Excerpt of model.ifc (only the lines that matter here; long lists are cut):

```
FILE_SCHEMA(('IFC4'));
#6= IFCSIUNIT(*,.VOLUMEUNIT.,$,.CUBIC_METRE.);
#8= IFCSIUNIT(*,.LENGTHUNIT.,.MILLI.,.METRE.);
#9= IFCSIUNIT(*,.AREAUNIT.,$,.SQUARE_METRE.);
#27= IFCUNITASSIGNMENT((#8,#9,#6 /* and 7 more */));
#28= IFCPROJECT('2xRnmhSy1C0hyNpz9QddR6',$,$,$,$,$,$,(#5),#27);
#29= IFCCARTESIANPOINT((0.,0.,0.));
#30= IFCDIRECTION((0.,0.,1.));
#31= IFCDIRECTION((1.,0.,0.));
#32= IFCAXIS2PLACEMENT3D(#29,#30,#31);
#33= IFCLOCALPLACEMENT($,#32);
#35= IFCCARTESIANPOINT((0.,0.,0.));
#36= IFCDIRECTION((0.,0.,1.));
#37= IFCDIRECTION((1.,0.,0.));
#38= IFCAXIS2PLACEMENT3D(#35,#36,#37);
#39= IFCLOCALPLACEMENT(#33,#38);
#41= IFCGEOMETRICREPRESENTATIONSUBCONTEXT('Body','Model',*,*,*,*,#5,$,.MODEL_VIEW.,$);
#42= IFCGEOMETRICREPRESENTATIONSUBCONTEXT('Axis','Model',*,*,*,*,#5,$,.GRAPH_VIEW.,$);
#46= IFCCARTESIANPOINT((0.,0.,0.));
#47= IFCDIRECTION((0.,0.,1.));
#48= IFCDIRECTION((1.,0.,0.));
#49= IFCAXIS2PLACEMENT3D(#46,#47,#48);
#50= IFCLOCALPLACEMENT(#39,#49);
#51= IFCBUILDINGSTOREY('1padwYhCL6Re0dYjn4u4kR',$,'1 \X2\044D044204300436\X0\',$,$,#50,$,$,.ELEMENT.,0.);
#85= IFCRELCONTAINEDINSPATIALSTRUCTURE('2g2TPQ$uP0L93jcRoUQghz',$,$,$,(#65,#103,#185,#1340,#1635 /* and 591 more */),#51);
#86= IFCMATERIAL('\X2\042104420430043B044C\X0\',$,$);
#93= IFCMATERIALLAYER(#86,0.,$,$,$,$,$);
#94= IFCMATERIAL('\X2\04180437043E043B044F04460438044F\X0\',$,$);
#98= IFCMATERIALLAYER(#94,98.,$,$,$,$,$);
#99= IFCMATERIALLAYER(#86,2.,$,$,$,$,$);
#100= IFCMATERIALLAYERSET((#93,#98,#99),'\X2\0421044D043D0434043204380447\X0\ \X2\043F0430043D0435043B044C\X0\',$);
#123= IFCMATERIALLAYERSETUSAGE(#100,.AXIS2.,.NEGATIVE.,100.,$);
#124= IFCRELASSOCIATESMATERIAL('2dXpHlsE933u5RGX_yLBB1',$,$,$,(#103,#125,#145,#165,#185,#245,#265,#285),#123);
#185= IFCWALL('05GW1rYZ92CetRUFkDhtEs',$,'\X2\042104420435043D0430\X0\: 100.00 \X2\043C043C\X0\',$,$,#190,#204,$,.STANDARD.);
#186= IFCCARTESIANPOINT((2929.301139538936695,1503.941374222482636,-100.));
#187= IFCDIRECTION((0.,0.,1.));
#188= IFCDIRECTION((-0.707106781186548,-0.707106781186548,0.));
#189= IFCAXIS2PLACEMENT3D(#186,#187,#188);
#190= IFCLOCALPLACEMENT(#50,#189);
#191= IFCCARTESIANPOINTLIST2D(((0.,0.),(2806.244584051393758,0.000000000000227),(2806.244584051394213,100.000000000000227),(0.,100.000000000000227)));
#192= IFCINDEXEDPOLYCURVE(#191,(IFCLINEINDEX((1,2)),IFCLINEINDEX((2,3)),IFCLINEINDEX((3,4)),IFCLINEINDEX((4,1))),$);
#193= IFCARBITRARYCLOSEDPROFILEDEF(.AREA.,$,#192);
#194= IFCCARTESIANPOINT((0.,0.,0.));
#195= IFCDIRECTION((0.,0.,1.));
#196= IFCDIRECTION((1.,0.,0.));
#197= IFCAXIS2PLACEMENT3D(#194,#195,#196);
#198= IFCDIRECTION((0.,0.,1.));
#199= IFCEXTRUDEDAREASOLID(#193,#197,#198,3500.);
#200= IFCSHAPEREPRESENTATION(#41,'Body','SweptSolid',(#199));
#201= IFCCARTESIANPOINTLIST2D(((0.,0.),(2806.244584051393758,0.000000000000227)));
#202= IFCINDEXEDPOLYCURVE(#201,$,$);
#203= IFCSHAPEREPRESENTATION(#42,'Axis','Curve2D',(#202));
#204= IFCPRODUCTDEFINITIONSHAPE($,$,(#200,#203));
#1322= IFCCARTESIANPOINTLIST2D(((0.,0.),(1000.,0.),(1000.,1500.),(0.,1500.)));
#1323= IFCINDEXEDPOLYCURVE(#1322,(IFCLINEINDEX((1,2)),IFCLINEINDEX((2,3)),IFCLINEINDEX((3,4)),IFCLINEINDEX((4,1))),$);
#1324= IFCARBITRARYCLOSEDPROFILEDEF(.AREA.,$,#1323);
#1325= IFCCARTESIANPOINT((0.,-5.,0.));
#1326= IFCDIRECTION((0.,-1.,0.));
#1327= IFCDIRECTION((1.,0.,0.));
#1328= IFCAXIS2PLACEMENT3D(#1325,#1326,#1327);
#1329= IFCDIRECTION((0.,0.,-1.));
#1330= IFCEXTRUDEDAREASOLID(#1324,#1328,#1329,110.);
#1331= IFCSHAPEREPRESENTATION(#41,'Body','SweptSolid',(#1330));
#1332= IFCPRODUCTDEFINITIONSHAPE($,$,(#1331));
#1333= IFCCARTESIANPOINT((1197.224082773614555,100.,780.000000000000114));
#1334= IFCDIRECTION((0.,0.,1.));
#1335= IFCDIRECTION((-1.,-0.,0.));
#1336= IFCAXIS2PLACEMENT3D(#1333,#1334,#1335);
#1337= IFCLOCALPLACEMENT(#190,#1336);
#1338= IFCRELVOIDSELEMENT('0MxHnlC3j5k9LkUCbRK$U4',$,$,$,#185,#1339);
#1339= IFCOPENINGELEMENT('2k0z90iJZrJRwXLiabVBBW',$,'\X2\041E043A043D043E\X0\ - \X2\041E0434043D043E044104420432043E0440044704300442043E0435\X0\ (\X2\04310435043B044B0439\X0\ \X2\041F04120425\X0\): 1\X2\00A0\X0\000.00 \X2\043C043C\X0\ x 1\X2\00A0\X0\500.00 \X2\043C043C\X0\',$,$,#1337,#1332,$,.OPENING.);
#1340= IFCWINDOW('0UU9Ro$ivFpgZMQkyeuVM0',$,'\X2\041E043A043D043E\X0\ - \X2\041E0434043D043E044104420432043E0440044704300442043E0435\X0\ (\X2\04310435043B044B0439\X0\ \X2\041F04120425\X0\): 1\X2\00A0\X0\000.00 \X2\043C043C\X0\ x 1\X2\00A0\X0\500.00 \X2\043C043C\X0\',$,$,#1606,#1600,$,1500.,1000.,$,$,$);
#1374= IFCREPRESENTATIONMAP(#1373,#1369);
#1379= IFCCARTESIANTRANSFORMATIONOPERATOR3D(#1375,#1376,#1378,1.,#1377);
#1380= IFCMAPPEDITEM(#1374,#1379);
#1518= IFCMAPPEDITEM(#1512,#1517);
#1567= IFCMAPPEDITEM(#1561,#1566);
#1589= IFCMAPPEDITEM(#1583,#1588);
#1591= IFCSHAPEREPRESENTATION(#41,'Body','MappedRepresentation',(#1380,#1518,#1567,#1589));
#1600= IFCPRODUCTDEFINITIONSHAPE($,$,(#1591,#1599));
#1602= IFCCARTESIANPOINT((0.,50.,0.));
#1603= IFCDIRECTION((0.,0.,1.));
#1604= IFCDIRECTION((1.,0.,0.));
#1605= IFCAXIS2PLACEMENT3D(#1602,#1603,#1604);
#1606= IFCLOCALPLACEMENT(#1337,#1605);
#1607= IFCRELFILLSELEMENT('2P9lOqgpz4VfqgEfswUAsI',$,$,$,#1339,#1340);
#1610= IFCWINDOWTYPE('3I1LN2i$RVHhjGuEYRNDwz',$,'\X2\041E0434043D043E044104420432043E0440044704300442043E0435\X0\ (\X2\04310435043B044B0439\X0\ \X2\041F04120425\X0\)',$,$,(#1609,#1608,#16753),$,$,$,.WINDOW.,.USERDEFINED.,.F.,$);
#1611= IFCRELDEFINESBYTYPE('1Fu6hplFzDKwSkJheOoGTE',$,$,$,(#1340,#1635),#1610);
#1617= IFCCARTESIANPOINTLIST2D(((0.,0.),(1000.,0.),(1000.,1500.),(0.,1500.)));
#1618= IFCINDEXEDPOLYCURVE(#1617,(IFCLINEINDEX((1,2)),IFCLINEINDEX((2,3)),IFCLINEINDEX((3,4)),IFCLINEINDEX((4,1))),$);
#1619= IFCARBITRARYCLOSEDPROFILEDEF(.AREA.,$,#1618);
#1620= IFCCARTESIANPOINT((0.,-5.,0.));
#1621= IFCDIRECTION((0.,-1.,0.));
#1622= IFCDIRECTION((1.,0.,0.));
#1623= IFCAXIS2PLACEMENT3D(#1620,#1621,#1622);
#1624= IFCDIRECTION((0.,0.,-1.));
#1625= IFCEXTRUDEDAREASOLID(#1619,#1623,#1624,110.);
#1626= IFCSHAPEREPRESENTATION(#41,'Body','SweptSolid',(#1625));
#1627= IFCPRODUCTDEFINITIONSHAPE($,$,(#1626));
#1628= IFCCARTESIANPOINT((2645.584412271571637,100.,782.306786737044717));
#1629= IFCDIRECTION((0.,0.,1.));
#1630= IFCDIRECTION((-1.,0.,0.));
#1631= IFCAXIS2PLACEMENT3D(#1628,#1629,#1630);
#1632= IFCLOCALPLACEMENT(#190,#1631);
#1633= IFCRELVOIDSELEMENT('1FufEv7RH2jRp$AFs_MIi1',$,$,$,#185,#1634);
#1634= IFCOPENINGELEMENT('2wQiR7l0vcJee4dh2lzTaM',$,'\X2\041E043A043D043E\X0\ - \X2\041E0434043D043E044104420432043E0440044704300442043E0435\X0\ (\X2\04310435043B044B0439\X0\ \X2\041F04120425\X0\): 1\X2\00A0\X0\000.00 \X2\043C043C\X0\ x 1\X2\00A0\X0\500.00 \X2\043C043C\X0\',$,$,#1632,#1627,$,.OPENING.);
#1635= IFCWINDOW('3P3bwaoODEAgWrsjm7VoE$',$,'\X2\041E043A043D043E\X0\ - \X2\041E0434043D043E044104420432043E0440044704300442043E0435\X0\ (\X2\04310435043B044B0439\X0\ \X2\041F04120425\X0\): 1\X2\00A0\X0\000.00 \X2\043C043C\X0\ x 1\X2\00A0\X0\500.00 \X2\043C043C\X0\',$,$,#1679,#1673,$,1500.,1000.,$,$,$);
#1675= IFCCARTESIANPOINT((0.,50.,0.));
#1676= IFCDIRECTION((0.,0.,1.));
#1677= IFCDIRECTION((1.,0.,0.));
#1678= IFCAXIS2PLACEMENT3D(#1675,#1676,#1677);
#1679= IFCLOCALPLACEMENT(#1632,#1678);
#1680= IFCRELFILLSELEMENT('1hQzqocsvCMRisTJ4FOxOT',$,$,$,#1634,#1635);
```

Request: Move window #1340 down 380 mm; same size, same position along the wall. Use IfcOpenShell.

```python
import numpy as np
import ifcopenshell
import ifcopenshell.api.geometry
import ifcopenshell.util.placement
import ifcopenshell.util.unit

model = ifcopenshell.open("model.ifc")
unit_scale = ifcopenshell.util.unit.calculate_unit_scale(model)

window = model.by_id(1340)
opening = window.FillsVoids[0].RelatingOpeningElement
dz = -380.0

shift = np.array([0.0, 0.0, dz])
# The window is placed relative to its opening, so it follows when the opening moves.
matrix = ifcopenshell.util.placement.get_local_placement(opening.ObjectPlacement)
matrix[:3, 3] += shift
ifcopenshell.api.geometry.edit_object_placement(
    model, product=opening, matrix=matrix, is_si=False, should_transform_children=True
)

print(f"moved by {dz * unit_scale:+.3f} m")

model.write("model_rev.ifc")
```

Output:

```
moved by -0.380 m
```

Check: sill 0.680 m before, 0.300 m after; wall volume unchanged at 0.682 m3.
